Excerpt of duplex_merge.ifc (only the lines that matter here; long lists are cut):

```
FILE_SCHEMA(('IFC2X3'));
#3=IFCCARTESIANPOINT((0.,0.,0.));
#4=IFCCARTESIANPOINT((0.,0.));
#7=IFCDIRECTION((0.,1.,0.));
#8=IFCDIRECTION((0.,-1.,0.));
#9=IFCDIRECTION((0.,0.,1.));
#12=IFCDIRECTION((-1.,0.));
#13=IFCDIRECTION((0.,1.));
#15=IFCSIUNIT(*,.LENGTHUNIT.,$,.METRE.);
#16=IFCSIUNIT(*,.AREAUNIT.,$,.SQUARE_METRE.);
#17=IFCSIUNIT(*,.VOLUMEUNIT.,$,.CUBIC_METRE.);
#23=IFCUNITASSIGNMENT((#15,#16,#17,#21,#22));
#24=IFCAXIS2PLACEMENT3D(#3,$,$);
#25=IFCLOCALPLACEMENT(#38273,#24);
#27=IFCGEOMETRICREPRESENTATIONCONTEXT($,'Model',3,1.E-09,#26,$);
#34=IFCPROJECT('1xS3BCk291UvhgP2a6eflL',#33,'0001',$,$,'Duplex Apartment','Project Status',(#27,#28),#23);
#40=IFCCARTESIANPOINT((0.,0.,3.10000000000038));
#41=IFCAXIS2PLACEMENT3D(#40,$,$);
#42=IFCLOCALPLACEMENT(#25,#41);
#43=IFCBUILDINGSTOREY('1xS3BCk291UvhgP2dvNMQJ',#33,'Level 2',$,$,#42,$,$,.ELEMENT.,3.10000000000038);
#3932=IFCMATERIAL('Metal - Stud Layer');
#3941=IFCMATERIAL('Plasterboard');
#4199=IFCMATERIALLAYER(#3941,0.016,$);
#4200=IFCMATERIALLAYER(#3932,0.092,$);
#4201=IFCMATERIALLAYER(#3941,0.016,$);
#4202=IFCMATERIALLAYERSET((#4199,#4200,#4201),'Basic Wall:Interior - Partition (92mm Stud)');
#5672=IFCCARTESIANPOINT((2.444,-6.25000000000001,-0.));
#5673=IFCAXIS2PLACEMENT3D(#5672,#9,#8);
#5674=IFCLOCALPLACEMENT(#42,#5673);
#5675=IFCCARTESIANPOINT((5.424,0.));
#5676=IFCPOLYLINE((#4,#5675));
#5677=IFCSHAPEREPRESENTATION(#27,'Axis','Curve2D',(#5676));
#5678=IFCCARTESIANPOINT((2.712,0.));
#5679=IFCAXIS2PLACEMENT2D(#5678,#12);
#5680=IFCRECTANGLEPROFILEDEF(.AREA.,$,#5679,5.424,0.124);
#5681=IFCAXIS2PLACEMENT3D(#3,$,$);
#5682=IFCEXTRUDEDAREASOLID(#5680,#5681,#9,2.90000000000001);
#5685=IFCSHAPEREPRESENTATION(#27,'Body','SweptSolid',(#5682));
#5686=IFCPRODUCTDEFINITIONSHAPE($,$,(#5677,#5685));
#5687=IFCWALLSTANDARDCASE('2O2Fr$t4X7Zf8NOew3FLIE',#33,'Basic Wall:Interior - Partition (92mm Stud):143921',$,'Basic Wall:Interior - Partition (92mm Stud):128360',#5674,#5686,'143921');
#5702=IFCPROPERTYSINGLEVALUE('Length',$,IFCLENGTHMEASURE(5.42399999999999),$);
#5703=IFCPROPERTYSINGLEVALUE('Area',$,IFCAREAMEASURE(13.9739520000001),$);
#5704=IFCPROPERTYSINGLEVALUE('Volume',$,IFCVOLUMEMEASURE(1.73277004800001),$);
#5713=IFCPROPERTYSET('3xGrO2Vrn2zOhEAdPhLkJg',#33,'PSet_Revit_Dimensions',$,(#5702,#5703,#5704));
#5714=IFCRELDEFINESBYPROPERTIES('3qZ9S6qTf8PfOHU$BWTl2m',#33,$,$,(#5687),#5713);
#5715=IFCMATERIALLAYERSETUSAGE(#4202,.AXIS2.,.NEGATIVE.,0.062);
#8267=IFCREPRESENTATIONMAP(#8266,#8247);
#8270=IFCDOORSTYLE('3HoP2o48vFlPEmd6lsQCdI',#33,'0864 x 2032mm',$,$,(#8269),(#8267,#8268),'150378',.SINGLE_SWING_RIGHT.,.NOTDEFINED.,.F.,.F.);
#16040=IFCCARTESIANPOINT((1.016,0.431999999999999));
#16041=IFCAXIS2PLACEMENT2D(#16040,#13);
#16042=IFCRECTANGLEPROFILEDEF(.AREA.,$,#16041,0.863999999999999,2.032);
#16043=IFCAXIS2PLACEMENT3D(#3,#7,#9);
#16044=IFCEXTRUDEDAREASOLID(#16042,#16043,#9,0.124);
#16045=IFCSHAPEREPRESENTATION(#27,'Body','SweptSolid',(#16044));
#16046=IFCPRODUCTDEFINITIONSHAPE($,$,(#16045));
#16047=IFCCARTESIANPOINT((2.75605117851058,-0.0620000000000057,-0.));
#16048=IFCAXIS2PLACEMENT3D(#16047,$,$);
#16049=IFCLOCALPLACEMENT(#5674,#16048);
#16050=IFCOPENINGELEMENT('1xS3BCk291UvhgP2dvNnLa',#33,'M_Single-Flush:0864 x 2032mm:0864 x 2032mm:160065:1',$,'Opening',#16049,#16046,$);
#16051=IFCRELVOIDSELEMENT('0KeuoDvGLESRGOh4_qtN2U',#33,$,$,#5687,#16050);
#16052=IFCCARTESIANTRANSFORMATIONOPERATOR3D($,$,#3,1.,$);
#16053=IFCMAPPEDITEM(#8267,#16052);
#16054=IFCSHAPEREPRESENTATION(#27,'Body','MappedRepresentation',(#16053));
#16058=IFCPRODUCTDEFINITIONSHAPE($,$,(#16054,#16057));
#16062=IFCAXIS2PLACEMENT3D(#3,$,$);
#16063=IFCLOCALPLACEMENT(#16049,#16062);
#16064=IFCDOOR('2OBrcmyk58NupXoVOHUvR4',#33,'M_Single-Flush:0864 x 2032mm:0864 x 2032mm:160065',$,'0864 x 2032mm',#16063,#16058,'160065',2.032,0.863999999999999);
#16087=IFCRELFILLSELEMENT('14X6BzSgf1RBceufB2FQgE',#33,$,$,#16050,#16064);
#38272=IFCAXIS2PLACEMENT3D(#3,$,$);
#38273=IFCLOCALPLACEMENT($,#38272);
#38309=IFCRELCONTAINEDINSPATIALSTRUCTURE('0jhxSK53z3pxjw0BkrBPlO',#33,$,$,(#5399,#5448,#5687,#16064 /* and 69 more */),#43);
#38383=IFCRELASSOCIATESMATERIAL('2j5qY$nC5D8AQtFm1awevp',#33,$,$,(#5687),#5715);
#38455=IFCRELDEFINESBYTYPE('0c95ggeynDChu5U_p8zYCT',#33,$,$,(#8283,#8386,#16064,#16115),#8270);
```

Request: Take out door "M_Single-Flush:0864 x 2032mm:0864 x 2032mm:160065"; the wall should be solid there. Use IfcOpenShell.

```python
import ifcopenshell
import ifcopenshell.api.feature
import ifcopenshell.api.pset
import ifcopenshell.api.root
import ifcopenshell.geom
import ifcopenshell.util.element
import ifcopenshell.util.shape
import ifcopenshell.util.unit

model = ifcopenshell.open("duplex_merge.ifc")
area_scale = ifcopenshell.util.unit.calculate_unit_scale(model, "AREAUNIT")
volume_scale = ifcopenshell.util.unit.calculate_unit_scale(model, "VOLUMEUNIT")
settings = ifcopenshell.geom.settings()


def volume(element):
    """Net volume in cubic metres, openings subtracted."""
    shape = ifcopenshell.geom.create_shape(settings, element)
    return ifcopenshell.util.shape.get_volume(shape.geometry)


door = model.by_id(16064)
opening = door.FillsVoids[0].RelatingOpeningElement
wall = opening.VoidsElements[0].RelatingBuildingElement
before = volume(wall)

ifcopenshell.api.root.remove_product(model, product=door)
ifcopenshell.api.feature.remove_feature(model, feature=opening)

after = volume(wall)
thickness = 0.124  # wall thickness in metres

# Update the wall's stored quantities.
pset = model.by_id(ifcopenshell.util.element.get_pset(wall, "PSet_Revit_Dimensions", should_inherit=False)["id"])
ifcopenshell.api.pset.edit_pset(model, pset=pset, properties={
    "Area": model.create_entity("IfcAreaMeasure", after / thickness / area_scale),
    "Volume": model.create_entity("IfcVolumeMeasure", after / volume_scale),
})

print(f"wall volume {before:.3f} -> {after:.3f} m3")

model.write("duplex_merge_rev.ifc")
```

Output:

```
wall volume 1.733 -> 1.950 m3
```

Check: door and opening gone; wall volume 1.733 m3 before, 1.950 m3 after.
